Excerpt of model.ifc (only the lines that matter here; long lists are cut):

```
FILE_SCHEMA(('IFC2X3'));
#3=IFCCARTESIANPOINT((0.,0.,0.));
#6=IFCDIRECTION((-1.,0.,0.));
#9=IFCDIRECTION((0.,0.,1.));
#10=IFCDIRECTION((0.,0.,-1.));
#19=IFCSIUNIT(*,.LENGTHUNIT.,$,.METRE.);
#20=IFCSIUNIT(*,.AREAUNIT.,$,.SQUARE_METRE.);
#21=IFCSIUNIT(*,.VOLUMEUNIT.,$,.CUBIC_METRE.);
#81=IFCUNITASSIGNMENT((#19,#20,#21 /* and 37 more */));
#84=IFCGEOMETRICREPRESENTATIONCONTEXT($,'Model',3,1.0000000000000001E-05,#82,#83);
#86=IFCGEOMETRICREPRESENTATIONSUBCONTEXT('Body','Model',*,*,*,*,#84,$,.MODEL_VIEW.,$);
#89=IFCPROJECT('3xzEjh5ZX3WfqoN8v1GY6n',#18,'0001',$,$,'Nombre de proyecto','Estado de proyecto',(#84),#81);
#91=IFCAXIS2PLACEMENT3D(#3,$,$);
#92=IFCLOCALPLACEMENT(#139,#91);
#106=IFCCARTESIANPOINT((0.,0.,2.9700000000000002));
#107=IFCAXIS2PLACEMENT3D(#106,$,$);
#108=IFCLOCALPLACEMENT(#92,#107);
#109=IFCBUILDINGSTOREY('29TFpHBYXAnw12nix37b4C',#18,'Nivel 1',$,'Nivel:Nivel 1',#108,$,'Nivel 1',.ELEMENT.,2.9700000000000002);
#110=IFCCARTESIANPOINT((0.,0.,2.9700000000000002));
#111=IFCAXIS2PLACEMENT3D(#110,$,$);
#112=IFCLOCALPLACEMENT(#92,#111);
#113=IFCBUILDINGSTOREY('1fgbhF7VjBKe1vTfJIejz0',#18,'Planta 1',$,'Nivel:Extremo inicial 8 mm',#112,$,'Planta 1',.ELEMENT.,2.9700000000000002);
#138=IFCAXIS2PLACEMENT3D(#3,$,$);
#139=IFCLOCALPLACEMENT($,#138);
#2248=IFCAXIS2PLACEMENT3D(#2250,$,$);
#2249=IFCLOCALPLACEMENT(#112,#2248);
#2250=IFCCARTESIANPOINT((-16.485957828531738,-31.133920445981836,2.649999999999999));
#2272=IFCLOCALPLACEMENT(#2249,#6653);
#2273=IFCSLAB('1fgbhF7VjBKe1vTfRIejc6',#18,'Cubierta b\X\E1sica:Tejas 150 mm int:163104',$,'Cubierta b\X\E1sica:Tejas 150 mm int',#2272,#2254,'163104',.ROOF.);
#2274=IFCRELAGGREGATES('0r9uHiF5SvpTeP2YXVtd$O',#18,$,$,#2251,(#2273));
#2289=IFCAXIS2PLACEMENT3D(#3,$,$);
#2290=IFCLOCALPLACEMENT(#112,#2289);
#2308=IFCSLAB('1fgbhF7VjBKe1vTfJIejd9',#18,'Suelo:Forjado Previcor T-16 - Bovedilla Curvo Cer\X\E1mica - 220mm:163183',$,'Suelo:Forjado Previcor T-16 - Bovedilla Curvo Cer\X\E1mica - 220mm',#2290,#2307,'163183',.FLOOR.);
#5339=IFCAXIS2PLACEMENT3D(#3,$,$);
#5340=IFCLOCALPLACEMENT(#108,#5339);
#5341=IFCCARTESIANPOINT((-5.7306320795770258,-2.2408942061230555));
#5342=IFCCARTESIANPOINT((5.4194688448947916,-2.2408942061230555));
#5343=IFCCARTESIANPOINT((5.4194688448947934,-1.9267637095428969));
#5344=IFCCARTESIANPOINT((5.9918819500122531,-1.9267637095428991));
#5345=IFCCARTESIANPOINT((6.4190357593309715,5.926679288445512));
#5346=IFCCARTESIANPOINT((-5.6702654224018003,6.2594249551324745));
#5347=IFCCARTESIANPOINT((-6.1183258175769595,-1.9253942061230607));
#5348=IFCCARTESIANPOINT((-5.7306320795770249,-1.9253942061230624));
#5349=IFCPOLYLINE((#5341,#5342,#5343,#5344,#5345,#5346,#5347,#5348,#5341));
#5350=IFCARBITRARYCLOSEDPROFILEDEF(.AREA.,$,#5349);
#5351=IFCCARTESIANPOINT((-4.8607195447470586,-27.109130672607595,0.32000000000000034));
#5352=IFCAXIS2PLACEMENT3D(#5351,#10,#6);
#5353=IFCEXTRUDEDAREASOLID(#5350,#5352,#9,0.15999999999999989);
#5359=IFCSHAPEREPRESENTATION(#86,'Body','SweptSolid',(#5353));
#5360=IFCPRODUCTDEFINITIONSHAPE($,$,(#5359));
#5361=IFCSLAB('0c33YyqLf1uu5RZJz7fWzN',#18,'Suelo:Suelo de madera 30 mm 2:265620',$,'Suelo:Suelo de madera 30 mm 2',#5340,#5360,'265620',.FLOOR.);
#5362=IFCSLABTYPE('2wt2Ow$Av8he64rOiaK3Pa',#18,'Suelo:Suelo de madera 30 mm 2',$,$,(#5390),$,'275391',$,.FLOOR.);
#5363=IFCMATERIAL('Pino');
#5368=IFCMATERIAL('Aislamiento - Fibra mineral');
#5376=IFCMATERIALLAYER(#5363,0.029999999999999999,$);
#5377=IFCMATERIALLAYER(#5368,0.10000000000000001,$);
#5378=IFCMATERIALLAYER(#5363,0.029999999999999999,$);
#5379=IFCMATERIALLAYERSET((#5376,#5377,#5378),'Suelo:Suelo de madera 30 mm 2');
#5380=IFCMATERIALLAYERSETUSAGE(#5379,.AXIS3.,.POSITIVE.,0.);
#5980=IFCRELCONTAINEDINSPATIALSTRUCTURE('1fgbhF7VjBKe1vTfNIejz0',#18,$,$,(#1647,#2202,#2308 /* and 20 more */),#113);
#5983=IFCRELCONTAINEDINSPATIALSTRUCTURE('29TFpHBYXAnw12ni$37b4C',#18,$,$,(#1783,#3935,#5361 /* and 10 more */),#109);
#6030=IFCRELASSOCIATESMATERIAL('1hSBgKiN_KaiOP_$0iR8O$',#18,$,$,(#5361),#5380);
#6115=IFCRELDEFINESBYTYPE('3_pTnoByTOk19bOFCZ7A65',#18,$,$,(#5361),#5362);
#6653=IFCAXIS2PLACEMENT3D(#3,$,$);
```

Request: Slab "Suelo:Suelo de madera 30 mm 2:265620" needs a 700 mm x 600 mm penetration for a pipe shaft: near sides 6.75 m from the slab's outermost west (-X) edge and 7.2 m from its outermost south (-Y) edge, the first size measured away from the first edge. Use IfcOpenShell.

```python
import numpy as np
import ifcopenshell
import ifcopenshell.api.feature
import ifcopenshell.api.geometry
import ifcopenshell.api.root
import ifcopenshell.geom
import ifcopenshell.util.placement
import ifcopenshell.util.representation
import ifcopenshell.util.shape
import ifcopenshell.util.unit

model = ifcopenshell.open("model.ifc")
unit_scale = ifcopenshell.util.unit.calculate_unit_scale(model)
settings = ifcopenshell.geom.settings()


def volume(element):
    """Net volume in cubic metres, openings subtracted."""
    shape = ifcopenshell.geom.create_shape(settings, element)
    return ifcopenshell.util.shape.get_volume(shape.geometry)


slab = model.by_guid("0c33YyqLf1uu5RZJz7fWzN")
before = volume(slab)

# Extent in the slab's own axes, in metres. The edges named are its -X and -Y sides.
slab_shape = ifcopenshell.geom.create_shape(settings, slab)
vertices = ifcopenshell.util.shape.get_vertices(slab_shape.geometry)
x_min, y_min, bottom = vertices.min(axis=0)
top = vertices[:, 2].max()

opening = ifcopenshell.api.root.create_entity(model, ifc_class="IfcOpeningElement", name="Pipe shaft opening")
context = ifcopenshell.util.representation.get_context(model, "Model", "Body", "MODEL_VIEW")
width, depth = 0.7, 0.6
outline = [(0.0, 0.0), (width, 0.0), (width, depth), (0.0, depth), (0.0, 0.0)]
# Overshoot both faces by 50 mm so the cut is clean.
shape = ifcopenshell.api.geometry.add_slab_representation(
    model, context=context, depth=top - bottom + 0.1, polyline=outline
)
ifcopenshell.api.geometry.assign_representation(model, product=opening, representation=shape)

matrix = ifcopenshell.util.placement.get_local_placement(slab.ObjectPlacement)
matrix[:, 3] = matrix @ np.append(np.array([x_min + 6.75, y_min + 7.2, bottom - 0.05]) / unit_scale, 1.0)
ifcopenshell.api.geometry.edit_object_placement(model, product=opening, matrix=matrix, is_si=False)
ifcopenshell.api.feature.add_feature(model, feature=opening, element=slab)

after = volume(slab)

print(f"slab volume {before:.3f} -> {after:.3f} m3")

model.write("model_v2.ifc")
```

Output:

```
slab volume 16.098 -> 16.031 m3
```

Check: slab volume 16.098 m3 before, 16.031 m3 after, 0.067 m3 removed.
